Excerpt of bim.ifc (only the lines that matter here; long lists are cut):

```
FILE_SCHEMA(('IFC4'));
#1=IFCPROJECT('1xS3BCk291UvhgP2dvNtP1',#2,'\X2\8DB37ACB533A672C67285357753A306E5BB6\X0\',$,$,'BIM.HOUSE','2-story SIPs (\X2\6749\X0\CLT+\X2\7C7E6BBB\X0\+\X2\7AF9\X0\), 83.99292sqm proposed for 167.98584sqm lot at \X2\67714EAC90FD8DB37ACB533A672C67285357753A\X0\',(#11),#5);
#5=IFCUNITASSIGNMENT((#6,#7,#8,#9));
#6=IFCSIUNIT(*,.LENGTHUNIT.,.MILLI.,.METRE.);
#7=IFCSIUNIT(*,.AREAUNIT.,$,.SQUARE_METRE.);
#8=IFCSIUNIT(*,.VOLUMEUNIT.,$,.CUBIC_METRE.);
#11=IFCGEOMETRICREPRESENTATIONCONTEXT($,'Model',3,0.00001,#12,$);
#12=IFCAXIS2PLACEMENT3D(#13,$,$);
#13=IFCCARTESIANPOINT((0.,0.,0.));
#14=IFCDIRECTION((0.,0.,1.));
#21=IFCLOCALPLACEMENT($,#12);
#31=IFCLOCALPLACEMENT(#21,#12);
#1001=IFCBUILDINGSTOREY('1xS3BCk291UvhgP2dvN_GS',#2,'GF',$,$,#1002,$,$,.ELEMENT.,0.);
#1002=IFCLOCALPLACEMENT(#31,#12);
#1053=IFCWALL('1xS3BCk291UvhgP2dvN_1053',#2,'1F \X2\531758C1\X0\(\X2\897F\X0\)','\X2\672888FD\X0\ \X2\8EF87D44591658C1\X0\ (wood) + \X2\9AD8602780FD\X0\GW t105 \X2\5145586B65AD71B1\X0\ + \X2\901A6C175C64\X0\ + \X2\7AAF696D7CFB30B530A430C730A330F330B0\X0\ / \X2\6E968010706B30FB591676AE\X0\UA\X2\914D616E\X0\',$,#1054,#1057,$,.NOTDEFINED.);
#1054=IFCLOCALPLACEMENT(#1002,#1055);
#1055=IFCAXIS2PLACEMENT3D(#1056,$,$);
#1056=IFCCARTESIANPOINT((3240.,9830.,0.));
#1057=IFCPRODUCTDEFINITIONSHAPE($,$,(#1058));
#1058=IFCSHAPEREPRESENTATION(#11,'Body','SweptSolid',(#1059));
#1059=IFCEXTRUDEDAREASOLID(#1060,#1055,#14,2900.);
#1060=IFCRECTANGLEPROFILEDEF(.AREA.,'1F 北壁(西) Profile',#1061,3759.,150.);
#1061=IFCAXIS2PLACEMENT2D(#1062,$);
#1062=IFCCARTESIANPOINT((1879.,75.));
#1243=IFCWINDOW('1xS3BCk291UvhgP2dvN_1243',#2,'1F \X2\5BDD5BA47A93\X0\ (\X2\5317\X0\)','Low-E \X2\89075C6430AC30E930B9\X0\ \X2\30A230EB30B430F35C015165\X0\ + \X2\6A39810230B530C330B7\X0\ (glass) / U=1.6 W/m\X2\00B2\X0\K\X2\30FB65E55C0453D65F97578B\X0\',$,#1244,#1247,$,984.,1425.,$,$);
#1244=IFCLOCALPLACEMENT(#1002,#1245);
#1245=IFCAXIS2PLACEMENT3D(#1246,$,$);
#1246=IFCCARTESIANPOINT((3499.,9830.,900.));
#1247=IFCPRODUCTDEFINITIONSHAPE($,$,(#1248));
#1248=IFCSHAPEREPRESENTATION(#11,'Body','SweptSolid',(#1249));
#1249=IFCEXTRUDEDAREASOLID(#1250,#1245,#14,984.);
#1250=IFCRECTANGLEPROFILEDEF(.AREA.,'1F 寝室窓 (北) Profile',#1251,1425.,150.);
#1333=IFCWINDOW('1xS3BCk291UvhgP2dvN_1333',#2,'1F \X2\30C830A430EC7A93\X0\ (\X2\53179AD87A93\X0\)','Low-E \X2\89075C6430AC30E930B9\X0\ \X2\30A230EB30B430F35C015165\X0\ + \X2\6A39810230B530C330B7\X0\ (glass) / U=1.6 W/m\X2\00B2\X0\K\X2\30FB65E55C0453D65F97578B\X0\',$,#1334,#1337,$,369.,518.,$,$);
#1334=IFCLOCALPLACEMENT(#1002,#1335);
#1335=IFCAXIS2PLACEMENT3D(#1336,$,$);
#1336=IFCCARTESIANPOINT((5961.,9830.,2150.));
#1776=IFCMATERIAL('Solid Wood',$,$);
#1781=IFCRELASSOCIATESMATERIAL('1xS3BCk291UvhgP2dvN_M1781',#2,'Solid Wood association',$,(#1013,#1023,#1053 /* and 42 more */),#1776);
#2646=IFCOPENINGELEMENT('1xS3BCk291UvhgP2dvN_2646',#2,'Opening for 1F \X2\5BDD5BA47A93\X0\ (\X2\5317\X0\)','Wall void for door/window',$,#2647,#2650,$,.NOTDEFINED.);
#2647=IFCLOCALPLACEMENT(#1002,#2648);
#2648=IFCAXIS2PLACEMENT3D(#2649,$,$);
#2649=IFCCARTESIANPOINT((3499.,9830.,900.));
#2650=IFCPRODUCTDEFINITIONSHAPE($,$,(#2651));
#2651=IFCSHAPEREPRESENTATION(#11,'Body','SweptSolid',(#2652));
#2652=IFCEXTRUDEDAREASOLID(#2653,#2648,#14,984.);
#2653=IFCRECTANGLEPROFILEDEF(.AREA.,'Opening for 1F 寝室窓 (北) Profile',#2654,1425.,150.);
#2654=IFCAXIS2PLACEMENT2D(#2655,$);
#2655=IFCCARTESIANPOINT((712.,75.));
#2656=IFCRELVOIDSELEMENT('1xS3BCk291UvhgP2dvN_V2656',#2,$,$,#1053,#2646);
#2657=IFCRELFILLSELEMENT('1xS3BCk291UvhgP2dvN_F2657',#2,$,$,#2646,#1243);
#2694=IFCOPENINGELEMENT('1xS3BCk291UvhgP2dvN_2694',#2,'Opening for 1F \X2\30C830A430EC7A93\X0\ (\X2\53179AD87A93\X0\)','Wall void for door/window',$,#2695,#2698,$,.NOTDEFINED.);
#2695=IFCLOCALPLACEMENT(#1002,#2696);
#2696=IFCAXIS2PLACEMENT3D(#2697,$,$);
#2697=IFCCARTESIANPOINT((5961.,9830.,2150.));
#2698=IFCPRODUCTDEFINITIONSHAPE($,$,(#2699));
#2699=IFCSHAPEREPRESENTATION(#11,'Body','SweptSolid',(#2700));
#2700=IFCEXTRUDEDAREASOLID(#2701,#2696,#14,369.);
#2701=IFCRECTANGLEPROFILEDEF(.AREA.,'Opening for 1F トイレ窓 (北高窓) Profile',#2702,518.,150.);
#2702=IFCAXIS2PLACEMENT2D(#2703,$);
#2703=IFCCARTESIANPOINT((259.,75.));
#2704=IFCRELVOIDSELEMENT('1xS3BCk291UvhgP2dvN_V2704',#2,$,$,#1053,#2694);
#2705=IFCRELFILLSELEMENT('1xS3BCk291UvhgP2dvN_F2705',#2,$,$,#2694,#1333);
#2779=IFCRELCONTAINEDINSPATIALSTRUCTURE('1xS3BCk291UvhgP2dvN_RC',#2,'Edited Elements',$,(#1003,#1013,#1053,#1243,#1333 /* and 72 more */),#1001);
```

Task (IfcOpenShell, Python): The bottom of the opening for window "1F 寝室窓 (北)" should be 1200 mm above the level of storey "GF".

```python
import numpy as np
import ifcopenshell
import ifcopenshell.api.geometry
import ifcopenshell.geom
import ifcopenshell.util.element
import ifcopenshell.util.placement
import ifcopenshell.util.shape
import ifcopenshell.util.unit

model = ifcopenshell.open("bim.ifc")
unit_scale = ifcopenshell.util.unit.calculate_unit_scale(model)

window = model.by_guid("1xS3BCk291UvhgP2dvN_1243")
opening = window.FillsVoids[0].RelatingOpeningElement
storey = ifcopenshell.util.element.get_container(window, ifc_class="IfcBuildingStorey")
level = ifcopenshell.util.placement.get_local_placement(storey.ObjectPlacement)[2, 3]

# The opening's origin need not be at the sill, so measure its lowest point.
shape = ifcopenshell.geom.create_shape(ifcopenshell.geom.settings(), opening)
bottom = ifcopenshell.util.shape.get_shape_bottom_elevation(shape, shape.geometry) / unit_scale
dz = level + 1.2 / unit_scale - bottom

shift = np.array([0.0, 0.0, dz])
# The window is not placed relative to its opening, so move both.
for product in (opening, window):
    matrix = ifcopenshell.util.placement.get_local_placement(product.ObjectPlacement)
    matrix[:3, 3] += shift
    ifcopenshell.api.geometry.edit_object_placement(model, product=product, matrix=matrix, is_si=False)

print(f"moved by {dz * unit_scale:+.3f} m")

model.write("bim_v2.ifc")
```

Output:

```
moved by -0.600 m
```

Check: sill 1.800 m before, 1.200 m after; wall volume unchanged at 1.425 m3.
